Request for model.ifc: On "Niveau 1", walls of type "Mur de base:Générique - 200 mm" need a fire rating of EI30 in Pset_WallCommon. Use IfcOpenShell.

First a look at what the model holds.

```python
import ifcopenshell
import ifcopenshell.util.element

model = ifcopenshell.open("model.ifc")
print(model.schema)
storey = next(s for s in model.by_type("IfcBuildingStorey") if s.Name == "Niveau 1")
walls = [e for e in ifcopenshell.util.element.get_decomposition(storey) if e.is_a("IfcWall")]
seen = {}
for e in walls:
    element_type = ifcopenshell.util.element.get_type(e)
    key = (element_type.Name if element_type != e and element_type else None, ifcopenshell.util.element.get_pset(e, "Pset_WallCommon", "FireRating"))
    seen[key] = seen.get(key, 0) + 1
for (name, value), count in sorted(seen.items(), key=str):
    print(count, "x", name, "|", value)
```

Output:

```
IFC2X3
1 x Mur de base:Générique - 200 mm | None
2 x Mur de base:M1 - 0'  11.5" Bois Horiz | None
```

```python
import ifcopenshell
import ifcopenshell.api.pset
import ifcopenshell.util.element

model = ifcopenshell.open("model.ifc")

storey = next(s for s in model.by_type("IfcBuildingStorey") if s.Name == "Niveau 1")
walls = [e for e in ifcopenshell.util.element.get_decomposition(storey) if e.is_a("IfcWall")]

count = 0
for e in walls:
    element_type = ifcopenshell.util.element.get_type(e)
    if element_type in (None, e) or element_type.Name != "Mur de base:Générique - 200 mm":
        continue
    # add_pset returns the element's existing set when there is one.
    pset = ifcopenshell.api.pset.add_pset(model, product=e, name="Pset_WallCommon")
    ifcopenshell.api.pset.edit_pset(model, pset=pset, properties={"FireRating": "EI30"})
    count += 1

print(count, "walls updated")

model.write("model_edited.ifc")
```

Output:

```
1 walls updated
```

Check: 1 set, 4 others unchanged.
